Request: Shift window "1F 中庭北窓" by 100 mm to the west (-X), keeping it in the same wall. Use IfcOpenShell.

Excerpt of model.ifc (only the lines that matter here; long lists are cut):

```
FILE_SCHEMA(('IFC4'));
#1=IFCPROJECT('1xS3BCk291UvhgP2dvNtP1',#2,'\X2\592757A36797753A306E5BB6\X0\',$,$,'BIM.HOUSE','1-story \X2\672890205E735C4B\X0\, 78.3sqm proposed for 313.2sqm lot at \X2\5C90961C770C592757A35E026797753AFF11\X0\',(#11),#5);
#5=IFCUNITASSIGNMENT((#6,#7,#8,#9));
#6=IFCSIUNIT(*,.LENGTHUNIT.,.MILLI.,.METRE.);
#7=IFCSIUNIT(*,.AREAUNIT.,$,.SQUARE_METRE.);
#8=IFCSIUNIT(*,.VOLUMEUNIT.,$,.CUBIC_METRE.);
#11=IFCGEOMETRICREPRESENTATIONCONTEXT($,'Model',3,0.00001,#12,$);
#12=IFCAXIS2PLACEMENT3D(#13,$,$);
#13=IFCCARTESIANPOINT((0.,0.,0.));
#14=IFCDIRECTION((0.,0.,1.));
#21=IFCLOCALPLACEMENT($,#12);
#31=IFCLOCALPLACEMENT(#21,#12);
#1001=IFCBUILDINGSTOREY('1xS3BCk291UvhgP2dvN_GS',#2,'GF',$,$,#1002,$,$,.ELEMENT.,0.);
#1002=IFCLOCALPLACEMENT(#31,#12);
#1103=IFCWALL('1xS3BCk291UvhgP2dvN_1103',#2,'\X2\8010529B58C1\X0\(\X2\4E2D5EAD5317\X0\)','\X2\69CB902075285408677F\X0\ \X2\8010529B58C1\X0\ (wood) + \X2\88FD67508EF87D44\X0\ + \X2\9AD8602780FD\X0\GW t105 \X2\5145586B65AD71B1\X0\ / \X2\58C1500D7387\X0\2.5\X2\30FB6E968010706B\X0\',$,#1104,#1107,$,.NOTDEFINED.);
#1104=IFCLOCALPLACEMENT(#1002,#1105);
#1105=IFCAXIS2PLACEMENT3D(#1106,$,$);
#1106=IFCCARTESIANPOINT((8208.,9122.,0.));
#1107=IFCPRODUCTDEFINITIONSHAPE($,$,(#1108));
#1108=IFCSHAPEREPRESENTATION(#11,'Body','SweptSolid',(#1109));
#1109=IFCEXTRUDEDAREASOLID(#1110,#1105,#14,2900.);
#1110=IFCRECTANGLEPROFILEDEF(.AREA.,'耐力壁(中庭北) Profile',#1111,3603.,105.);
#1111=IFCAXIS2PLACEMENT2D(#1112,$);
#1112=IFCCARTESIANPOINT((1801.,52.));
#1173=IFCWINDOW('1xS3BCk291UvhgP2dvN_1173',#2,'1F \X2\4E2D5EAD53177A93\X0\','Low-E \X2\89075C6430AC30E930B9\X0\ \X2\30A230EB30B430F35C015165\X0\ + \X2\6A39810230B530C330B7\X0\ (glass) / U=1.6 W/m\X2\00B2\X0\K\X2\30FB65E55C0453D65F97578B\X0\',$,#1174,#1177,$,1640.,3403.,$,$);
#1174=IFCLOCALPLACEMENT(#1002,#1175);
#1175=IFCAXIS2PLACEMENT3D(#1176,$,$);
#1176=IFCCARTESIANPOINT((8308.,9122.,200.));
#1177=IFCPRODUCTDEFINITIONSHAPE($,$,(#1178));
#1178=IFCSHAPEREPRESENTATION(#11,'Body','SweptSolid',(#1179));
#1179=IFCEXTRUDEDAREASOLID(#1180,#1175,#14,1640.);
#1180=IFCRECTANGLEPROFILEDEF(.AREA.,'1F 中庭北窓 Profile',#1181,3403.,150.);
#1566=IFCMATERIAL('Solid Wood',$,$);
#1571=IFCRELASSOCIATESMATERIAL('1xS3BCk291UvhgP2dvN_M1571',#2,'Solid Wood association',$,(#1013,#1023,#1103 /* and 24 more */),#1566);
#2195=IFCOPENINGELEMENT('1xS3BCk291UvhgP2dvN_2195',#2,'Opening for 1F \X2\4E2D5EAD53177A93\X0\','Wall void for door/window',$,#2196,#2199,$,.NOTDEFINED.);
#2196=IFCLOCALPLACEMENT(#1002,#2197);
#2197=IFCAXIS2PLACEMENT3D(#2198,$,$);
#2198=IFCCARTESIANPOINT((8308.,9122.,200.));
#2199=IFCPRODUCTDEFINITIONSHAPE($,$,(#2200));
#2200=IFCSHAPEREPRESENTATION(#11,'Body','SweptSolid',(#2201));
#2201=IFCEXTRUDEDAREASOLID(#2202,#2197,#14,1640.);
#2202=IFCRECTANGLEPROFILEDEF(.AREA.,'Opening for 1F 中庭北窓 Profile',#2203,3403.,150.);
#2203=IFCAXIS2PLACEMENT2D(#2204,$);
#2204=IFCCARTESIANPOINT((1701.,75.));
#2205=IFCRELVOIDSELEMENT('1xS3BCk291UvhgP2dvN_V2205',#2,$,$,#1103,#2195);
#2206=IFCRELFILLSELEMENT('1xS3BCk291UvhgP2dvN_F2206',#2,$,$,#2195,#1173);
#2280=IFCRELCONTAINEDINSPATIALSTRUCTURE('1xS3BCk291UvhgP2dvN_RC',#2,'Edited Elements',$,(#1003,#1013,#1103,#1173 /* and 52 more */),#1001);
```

```python
import ifcopenshell
import ifcopenshell.api.geometry
import ifcopenshell.util.placement
import ifcopenshell.util.unit

model = ifcopenshell.open("model.ifc")
unit_scale = ifcopenshell.util.unit.calculate_unit_scale(model)

window = model.by_id(1173)
opening = window.FillsVoids[0].RelatingOpeningElement
wall = opening.VoidsElements[0].RelatingBuildingElement

wall_matrix = ifcopenshell.util.placement.get_local_placement(wall.ObjectPlacement)
shift = wall_matrix[:3, 0] * -0.1 / unit_scale
before = ifcopenshell.util.placement.get_local_placement(window.ObjectPlacement)[:3, 3].copy()

# The window is not placed relative to its opening, so move both.
for product in (opening, window):
    matrix = ifcopenshell.util.placement.get_local_placement(product.ObjectPlacement)
    matrix[:3, 3] += shift
    ifcopenshell.api.geometry.edit_object_placement(model, product=product, matrix=matrix, is_si=False)

after = ifcopenshell.util.placement.get_local_placement(window.ObjectPlacement)[:3, 3]
print("window moved by", (after - before).round(3) + 0.0)

model.write("model_v2.ifc")
```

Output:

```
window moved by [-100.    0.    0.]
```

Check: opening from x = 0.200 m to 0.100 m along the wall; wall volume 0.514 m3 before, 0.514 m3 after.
